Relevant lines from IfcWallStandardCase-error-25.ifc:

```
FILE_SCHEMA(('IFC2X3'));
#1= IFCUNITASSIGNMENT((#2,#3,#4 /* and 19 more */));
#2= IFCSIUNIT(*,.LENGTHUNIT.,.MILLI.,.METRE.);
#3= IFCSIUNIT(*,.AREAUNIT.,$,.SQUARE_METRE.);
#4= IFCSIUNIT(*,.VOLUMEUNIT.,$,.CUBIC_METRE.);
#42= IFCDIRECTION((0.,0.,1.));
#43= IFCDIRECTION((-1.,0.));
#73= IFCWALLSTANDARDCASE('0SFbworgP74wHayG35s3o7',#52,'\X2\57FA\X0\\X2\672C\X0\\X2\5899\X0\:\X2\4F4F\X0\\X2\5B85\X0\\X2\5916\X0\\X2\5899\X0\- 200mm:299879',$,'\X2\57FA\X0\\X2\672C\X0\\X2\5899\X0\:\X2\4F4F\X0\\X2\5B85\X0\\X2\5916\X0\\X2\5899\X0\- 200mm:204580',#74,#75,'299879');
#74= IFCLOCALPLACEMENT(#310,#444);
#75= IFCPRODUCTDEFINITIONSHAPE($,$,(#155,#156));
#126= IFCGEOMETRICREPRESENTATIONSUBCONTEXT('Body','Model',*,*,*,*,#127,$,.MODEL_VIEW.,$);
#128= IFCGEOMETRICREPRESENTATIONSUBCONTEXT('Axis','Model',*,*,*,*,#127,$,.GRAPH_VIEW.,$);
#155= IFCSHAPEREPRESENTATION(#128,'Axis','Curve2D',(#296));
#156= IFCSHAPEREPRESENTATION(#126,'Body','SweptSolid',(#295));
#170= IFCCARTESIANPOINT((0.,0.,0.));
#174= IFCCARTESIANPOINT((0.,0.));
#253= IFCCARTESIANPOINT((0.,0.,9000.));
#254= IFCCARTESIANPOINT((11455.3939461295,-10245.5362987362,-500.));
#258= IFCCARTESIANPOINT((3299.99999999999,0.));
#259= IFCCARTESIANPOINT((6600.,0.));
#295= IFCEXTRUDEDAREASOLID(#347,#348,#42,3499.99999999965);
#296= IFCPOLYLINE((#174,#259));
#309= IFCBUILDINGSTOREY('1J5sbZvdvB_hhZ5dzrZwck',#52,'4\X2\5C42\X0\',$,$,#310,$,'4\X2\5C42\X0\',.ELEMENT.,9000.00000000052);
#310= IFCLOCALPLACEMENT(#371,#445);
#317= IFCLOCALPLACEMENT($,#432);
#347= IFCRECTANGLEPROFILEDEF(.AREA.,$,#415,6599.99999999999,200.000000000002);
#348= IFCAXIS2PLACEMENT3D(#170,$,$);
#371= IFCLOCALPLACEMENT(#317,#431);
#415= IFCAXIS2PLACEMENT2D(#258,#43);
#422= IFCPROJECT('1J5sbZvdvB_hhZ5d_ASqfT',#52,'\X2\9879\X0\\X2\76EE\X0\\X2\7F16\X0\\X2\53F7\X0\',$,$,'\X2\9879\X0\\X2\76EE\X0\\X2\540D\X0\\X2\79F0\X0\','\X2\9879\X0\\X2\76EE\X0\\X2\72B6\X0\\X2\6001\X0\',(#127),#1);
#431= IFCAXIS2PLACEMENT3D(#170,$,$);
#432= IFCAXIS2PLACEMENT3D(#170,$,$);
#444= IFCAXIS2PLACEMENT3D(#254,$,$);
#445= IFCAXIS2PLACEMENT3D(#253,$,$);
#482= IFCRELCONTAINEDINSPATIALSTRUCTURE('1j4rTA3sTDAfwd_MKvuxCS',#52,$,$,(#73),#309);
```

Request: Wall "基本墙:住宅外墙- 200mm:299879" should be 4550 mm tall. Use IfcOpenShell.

```python
import ifcopenshell
import ifcopenshell.geom
import ifcopenshell.util.representation
import ifcopenshell.util.shape
import ifcopenshell.util.unit

model = ifcopenshell.open("IfcWallStandardCase-error-25.ifc")
unit_scale = ifcopenshell.util.unit.calculate_unit_scale(model)
settings = ifcopenshell.geom.settings()


def volume(element):
    """Net volume in cubic metres, openings subtracted."""
    shape = ifcopenshell.geom.create_shape(settings, element)
    return ifcopenshell.util.shape.get_volume(shape.geometry)


wall = model.by_guid("0SFbworgP74wHayG35s3o7")
before = volume(wall)

body = ifcopenshell.util.representation.get_representation(wall, "Model", "Body")
solid = body.Items[0]
old_height = solid.Depth
solid.Depth = 4.55 / unit_scale
after = volume(wall)

print(f"height {old_height:g} -> {solid.Depth:g}, volume {before:.3f} -> {after:.3f} m3")

model.write("IfcWallStandardCase-error-25_updated.ifc")
```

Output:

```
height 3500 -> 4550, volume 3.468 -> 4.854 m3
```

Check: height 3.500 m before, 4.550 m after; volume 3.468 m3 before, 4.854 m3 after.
